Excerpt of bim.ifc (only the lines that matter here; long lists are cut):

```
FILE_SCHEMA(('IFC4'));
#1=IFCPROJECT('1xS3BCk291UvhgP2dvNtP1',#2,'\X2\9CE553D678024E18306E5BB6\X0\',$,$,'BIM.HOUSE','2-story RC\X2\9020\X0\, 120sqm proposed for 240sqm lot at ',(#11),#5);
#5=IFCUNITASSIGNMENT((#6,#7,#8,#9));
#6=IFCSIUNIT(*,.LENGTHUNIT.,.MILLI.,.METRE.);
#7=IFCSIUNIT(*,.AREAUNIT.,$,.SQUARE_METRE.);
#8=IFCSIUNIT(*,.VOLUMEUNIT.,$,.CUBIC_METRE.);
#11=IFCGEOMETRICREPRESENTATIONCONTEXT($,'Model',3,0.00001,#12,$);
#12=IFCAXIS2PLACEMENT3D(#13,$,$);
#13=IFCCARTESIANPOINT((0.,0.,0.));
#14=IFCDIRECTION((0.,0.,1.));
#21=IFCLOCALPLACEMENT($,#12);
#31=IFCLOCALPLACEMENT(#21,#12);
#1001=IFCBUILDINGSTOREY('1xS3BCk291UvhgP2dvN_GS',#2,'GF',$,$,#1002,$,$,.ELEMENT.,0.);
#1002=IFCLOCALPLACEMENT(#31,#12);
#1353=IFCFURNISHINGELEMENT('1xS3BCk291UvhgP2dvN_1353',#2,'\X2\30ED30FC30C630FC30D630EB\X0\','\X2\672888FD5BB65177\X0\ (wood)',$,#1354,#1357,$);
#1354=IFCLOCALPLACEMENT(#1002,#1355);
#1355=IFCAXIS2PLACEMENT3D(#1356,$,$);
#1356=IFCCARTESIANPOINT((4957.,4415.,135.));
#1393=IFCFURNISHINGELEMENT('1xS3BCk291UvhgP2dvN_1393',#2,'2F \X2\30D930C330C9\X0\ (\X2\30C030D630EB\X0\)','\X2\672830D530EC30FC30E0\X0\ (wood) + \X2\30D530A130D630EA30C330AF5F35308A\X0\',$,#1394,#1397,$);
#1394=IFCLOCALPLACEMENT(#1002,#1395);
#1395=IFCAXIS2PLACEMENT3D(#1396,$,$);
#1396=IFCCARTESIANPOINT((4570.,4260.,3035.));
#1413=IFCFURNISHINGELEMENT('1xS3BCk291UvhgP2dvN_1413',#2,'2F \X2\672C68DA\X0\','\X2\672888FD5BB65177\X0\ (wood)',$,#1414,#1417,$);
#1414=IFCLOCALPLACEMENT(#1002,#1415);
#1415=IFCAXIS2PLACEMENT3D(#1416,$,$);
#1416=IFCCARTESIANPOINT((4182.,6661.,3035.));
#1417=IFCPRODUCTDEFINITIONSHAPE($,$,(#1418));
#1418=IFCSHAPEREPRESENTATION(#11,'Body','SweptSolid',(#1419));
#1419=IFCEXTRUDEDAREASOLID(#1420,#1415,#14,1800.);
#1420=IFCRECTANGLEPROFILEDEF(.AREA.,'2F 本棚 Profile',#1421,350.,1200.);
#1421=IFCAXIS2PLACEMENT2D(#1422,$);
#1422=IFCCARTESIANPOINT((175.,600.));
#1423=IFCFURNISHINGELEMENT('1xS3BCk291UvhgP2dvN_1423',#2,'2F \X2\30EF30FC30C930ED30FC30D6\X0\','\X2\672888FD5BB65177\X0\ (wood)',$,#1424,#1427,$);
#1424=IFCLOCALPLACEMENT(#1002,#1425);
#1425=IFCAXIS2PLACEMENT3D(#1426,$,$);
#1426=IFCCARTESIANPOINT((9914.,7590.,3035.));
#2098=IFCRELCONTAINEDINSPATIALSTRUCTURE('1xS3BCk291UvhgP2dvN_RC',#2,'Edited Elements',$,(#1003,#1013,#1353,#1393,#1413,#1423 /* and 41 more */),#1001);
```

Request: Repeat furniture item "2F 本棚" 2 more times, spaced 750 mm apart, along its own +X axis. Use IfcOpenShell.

```python
import ifcopenshell
import ifcopenshell.api.geometry
import ifcopenshell.api.root
import ifcopenshell.util.element
import ifcopenshell.util.placement
import ifcopenshell.util.unit

model = ifcopenshell.open("bim.ifc")
unit_scale = ifcopenshell.util.unit.calculate_unit_scale(model)


def reuse_history(source, copy):
    """copy_class also copies each property set's owner history, people and application; keep the originals."""
    for rel in copy.IsDefinedBy:
        if rel.is_a("IfcRelDefinesByProperties") and (history := rel.RelatingPropertyDefinition.OwnerHistory):
            rel.RelatingPropertyDefinition.OwnerHistory = source.OwnerHistory
            ifcopenshell.util.element.remove_deep2(model, history)


source = model.by_guid("1xS3BCk291UvhgP2dvN_1413")
base = ifcopenshell.util.placement.get_local_placement(source.ObjectPlacement)
step = base[:3, 0] * 0.75 / unit_scale

for i in range(1, 3):
    copy = ifcopenshell.api.root.copy_class(model, product=source)
    copy.Representation = ifcopenshell.util.element.copy_deep(
        model, source.Representation, exclude=["IfcGeometricRepresentationContext", "IfcRepresentationMap"]
    )
    reuse_history(source, copy)
    matrix = base.copy()
    matrix[:3, 3] += i * step
    print("added at", matrix[:3, 3].round(3) + 0.0)
    ifcopenshell.api.geometry.edit_object_placement(model, product=copy, matrix=matrix, is_si=False)

model.write("bim_v2.ifc")
```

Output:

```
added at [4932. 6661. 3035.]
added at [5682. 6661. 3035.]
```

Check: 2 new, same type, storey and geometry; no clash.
